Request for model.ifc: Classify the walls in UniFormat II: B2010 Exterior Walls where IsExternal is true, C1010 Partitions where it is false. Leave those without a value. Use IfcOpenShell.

First a look at what the model holds.

```python
import ifcopenshell
import ifcopenshell.util.element

model = ifcopenshell.open("model.ifc")
print(model.schema)
print("classifications:", [c.Name for c in model.by_type("IfcClassification")])
values = [ifcopenshell.util.element.get_pset(e, "Pset_WallCommon", "IsExternal") for e in model.by_type("IfcWall")]
for value in (True, False, None):
    print("IsExternal", value, values.count(value))
```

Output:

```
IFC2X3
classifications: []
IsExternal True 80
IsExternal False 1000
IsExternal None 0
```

```python
import ifcopenshell
import ifcopenshell.api.classification
import ifcopenshell.util.element

model = ifcopenshell.open("model.ifc")

# IFC2X3 requires Source and Edition and has no link from the project to the system.
system = model.create_entity("IfcClassification", Source="ASTM", Edition="E1557", Name="UniFormat II")

walls = model.by_type("IfcWall")
external = {e: ifcopenshell.util.element.get_pset(e, "Pset_WallCommon", "IsExternal") for e in walls}
for flag, code, name in ((True, "B2010", "Exterior Walls"), (False, "C1010", "Partitions")):
    products = [e for e in walls if external[e] is flag]
    ifcopenshell.api.classification.add_reference(
        model, products=products, classification=system, identification=code, name=name
    )
    print(code, len(products))

model.write("model_edited.ifc")
```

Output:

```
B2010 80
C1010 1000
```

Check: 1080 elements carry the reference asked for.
